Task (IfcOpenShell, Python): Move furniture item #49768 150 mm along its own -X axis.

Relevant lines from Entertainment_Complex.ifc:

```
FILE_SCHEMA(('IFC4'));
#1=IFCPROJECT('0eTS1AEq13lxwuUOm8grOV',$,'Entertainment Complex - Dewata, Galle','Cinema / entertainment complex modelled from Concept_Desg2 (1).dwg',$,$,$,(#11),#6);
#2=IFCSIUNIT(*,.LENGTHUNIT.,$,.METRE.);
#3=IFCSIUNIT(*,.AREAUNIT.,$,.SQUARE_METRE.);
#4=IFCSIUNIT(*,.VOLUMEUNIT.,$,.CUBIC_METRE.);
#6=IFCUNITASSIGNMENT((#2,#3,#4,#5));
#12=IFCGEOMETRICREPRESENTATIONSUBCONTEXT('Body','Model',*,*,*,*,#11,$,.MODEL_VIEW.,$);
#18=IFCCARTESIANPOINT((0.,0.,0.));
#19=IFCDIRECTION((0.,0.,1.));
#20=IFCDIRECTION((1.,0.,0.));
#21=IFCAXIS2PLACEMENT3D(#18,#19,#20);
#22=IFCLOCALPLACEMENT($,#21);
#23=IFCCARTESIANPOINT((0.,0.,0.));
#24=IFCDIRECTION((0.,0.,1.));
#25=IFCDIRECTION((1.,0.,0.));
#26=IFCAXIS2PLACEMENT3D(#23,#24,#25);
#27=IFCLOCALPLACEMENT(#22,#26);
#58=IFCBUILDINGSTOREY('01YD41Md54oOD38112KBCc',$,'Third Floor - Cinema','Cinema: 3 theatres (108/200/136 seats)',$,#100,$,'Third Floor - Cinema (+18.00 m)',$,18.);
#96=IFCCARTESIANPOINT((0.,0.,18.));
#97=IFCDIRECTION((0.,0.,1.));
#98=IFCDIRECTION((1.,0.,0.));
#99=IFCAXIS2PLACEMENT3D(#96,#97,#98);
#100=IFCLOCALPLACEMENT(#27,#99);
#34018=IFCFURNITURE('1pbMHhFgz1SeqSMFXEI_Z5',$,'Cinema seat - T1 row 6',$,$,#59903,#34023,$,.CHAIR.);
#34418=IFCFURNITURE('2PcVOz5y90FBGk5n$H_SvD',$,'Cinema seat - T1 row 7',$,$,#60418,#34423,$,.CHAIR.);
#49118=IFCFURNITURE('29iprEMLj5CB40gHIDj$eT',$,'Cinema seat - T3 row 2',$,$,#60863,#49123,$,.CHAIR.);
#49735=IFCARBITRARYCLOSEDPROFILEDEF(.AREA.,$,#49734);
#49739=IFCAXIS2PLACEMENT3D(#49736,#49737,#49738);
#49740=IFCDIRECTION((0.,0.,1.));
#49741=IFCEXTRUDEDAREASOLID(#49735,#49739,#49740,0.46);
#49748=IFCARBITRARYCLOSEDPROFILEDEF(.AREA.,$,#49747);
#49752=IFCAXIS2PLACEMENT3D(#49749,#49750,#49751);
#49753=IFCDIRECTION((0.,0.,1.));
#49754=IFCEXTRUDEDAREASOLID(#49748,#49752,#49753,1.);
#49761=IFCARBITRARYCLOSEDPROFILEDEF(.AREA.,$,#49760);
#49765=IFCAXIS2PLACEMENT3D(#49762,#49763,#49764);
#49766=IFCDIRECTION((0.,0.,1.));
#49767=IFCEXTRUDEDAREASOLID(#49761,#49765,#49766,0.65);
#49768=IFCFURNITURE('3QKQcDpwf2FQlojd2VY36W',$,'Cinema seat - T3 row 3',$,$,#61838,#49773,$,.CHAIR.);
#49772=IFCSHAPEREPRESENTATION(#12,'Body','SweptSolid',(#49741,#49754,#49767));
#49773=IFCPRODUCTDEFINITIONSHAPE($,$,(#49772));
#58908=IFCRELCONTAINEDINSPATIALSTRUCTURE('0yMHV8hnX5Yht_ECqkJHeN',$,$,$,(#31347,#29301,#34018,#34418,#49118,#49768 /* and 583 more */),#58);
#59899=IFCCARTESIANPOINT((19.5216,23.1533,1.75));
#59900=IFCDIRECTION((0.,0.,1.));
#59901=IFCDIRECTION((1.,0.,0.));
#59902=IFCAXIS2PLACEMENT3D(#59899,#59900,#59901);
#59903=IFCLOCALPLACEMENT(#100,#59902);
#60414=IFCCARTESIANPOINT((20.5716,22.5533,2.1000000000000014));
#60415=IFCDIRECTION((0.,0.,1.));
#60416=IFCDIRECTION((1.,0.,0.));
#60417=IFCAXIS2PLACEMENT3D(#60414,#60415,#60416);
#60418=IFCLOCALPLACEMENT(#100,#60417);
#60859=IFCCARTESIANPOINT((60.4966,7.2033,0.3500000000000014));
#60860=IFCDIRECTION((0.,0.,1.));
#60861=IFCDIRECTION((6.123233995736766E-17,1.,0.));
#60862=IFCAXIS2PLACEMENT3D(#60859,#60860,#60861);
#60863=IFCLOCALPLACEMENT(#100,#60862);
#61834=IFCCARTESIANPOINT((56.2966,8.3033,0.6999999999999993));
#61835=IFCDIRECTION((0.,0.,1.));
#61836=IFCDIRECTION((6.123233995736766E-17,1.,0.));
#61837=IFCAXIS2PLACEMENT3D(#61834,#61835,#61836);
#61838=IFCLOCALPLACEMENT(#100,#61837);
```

```python
import ifcopenshell
import ifcopenshell.api.geometry
import ifcopenshell.util.placement
import ifcopenshell.util.unit

model = ifcopenshell.open("Entertainment_Complex.ifc")
unit_scale = ifcopenshell.util.unit.calculate_unit_scale(model)

item = model.by_guid("3QKQcDpwf2FQlojd2VY36W")
matrix = ifcopenshell.util.placement.get_local_placement(item.ObjectPlacement)
matrix[:3, 3] -= matrix[:3, 0] * 0.15 / unit_scale
ifcopenshell.api.geometry.edit_object_placement(model, product=item, matrix=matrix, is_si=False)

print(ifcopenshell.util.placement.get_local_placement(item.ObjectPlacement).round(3) + 0.0)

model.write("Entertainment_Complex_v2.ifc")
```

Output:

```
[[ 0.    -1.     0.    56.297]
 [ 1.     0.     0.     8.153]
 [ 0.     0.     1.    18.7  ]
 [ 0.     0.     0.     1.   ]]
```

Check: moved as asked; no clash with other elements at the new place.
